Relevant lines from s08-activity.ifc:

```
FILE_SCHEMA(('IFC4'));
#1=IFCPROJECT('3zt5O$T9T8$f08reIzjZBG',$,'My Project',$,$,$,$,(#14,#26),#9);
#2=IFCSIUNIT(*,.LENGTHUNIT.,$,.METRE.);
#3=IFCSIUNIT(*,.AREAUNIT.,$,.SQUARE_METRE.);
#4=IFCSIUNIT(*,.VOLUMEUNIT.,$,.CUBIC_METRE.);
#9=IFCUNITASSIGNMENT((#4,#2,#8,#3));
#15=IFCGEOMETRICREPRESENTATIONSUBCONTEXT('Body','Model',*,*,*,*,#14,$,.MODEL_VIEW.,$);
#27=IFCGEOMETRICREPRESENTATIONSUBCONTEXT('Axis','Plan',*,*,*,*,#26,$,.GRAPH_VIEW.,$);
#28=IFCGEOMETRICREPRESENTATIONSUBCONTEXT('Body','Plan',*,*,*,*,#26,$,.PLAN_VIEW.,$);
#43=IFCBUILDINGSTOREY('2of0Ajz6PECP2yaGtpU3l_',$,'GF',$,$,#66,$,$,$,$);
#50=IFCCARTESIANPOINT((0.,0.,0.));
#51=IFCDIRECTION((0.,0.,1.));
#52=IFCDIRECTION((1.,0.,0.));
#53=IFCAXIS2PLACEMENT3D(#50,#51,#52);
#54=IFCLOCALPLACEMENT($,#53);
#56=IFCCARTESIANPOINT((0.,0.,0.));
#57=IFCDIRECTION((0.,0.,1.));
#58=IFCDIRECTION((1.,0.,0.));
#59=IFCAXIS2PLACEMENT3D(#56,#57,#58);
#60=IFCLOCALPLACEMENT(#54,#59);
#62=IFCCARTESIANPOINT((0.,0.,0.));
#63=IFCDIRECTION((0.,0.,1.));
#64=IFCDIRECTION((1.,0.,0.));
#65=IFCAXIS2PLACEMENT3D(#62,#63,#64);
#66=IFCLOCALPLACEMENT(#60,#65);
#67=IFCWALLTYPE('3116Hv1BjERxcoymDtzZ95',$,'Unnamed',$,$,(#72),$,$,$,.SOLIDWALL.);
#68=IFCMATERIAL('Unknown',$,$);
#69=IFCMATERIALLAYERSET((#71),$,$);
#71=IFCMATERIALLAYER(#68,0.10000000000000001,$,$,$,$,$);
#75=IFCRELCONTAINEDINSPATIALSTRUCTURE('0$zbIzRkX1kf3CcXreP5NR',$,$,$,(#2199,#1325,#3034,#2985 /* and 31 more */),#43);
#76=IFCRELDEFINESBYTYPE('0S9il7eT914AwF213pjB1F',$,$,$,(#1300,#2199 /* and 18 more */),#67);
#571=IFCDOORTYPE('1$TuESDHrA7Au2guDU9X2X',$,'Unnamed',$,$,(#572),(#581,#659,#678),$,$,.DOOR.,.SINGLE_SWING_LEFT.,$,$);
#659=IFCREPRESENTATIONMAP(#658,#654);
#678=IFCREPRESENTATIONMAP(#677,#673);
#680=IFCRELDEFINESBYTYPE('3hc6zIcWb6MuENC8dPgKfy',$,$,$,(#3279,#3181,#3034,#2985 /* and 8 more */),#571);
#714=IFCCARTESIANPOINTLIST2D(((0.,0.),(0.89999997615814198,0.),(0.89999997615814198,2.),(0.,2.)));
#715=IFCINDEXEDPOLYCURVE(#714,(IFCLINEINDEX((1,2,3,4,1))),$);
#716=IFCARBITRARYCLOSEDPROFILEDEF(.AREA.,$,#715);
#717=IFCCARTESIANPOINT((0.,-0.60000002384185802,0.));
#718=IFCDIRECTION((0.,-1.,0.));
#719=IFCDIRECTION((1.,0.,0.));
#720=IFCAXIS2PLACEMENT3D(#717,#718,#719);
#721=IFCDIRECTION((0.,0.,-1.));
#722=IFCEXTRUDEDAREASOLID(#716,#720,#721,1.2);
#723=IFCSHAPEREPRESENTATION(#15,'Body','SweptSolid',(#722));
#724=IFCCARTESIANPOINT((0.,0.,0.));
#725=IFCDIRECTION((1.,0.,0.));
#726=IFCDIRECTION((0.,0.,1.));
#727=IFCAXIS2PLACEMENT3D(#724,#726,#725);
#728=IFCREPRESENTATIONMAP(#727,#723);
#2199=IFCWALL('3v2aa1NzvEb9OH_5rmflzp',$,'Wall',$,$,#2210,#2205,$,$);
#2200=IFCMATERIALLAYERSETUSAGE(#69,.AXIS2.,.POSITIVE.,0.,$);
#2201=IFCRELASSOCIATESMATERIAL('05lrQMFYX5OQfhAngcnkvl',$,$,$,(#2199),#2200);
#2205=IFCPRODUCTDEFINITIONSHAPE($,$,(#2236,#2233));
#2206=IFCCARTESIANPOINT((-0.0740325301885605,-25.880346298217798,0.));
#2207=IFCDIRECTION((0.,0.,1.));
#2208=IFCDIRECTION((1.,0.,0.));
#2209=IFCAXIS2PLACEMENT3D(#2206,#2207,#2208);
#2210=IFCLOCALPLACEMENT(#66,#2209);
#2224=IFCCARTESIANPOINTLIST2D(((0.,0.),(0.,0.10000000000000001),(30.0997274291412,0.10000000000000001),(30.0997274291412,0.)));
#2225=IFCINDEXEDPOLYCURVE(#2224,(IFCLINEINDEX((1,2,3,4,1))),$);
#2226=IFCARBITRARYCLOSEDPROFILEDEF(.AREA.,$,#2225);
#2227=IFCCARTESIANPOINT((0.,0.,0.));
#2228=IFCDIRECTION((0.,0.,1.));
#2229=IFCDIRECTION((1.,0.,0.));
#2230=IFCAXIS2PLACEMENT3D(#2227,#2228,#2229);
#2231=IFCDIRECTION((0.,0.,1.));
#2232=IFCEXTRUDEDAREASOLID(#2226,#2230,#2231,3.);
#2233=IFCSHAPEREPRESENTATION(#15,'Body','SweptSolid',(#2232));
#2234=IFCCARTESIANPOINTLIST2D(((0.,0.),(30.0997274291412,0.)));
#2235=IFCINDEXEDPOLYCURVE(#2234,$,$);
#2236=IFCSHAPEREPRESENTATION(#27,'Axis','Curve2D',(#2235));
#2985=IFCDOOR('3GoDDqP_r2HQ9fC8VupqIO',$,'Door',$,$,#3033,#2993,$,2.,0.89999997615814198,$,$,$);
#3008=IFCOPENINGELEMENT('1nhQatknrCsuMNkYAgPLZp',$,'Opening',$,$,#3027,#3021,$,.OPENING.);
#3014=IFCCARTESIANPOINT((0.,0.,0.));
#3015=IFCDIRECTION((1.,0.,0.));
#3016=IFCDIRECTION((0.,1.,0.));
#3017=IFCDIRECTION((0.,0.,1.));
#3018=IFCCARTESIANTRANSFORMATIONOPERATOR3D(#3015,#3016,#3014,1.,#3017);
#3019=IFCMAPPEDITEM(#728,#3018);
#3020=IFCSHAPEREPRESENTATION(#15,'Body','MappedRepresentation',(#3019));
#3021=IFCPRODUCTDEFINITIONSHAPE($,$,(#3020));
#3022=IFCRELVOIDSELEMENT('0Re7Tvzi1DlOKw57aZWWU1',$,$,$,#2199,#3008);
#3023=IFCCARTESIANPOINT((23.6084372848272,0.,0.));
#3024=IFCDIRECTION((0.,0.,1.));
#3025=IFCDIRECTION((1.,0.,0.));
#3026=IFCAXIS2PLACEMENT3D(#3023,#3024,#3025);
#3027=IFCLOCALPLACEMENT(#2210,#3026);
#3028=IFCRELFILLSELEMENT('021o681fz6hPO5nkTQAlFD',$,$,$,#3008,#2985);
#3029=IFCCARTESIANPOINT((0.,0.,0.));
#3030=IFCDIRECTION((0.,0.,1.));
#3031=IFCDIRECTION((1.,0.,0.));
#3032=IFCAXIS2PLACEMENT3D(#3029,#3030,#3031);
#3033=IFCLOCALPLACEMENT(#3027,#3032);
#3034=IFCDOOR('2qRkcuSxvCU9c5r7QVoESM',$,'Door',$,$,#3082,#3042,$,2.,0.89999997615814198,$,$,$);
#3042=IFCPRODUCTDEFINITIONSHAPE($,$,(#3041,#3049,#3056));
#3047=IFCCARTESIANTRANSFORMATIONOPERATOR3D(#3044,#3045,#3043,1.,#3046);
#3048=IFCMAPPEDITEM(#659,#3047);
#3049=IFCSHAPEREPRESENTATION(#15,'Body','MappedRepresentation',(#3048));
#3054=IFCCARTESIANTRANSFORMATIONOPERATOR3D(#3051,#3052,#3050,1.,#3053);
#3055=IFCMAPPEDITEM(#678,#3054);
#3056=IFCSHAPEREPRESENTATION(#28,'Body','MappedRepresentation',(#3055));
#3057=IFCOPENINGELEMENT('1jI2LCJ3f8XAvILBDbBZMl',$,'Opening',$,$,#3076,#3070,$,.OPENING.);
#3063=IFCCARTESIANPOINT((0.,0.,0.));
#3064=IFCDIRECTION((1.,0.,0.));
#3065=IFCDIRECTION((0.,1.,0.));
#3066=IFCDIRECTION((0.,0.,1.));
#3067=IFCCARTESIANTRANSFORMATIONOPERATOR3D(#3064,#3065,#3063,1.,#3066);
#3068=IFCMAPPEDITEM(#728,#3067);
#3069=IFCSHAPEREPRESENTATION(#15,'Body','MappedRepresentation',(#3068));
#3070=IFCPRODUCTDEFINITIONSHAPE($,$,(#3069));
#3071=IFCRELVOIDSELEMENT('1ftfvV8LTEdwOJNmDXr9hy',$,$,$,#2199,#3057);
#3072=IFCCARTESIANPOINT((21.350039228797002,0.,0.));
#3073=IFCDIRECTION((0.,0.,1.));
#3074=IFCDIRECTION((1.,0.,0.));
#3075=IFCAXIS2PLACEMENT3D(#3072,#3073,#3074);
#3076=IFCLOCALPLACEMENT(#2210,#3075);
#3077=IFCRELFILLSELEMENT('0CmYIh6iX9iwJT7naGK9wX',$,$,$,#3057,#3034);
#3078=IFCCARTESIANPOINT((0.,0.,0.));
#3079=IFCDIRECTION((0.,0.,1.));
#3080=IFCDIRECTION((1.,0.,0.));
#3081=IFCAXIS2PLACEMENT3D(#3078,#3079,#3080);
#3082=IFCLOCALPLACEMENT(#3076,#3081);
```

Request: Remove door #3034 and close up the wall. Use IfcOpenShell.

```python
import ifcopenshell
import ifcopenshell.api.feature
import ifcopenshell.api.root
import ifcopenshell.geom
import ifcopenshell.util.shape

model = ifcopenshell.open("s08-activity.ifc")
settings = ifcopenshell.geom.settings()


def volume(element):
    """Net volume in cubic metres, openings subtracted."""
    shape = ifcopenshell.geom.create_shape(settings, element)
    return ifcopenshell.util.shape.get_volume(shape.geometry)


door = model.by_guid("2qRkcuSxvCU9c5r7QVoESM")
opening = door.FillsVoids[0].RelatingOpeningElement
wall = opening.VoidsElements[0].RelatingBuildingElement
before = volume(wall)

ifcopenshell.api.root.remove_product(model, product=door)
ifcopenshell.api.feature.remove_feature(model, feature=opening)

after = volume(wall)

print(f"wall volume {before:.3f} -> {after:.3f} m3")

model.write("s08-activity_rev.ifc")
```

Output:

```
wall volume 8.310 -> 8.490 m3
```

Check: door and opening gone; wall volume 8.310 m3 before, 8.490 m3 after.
